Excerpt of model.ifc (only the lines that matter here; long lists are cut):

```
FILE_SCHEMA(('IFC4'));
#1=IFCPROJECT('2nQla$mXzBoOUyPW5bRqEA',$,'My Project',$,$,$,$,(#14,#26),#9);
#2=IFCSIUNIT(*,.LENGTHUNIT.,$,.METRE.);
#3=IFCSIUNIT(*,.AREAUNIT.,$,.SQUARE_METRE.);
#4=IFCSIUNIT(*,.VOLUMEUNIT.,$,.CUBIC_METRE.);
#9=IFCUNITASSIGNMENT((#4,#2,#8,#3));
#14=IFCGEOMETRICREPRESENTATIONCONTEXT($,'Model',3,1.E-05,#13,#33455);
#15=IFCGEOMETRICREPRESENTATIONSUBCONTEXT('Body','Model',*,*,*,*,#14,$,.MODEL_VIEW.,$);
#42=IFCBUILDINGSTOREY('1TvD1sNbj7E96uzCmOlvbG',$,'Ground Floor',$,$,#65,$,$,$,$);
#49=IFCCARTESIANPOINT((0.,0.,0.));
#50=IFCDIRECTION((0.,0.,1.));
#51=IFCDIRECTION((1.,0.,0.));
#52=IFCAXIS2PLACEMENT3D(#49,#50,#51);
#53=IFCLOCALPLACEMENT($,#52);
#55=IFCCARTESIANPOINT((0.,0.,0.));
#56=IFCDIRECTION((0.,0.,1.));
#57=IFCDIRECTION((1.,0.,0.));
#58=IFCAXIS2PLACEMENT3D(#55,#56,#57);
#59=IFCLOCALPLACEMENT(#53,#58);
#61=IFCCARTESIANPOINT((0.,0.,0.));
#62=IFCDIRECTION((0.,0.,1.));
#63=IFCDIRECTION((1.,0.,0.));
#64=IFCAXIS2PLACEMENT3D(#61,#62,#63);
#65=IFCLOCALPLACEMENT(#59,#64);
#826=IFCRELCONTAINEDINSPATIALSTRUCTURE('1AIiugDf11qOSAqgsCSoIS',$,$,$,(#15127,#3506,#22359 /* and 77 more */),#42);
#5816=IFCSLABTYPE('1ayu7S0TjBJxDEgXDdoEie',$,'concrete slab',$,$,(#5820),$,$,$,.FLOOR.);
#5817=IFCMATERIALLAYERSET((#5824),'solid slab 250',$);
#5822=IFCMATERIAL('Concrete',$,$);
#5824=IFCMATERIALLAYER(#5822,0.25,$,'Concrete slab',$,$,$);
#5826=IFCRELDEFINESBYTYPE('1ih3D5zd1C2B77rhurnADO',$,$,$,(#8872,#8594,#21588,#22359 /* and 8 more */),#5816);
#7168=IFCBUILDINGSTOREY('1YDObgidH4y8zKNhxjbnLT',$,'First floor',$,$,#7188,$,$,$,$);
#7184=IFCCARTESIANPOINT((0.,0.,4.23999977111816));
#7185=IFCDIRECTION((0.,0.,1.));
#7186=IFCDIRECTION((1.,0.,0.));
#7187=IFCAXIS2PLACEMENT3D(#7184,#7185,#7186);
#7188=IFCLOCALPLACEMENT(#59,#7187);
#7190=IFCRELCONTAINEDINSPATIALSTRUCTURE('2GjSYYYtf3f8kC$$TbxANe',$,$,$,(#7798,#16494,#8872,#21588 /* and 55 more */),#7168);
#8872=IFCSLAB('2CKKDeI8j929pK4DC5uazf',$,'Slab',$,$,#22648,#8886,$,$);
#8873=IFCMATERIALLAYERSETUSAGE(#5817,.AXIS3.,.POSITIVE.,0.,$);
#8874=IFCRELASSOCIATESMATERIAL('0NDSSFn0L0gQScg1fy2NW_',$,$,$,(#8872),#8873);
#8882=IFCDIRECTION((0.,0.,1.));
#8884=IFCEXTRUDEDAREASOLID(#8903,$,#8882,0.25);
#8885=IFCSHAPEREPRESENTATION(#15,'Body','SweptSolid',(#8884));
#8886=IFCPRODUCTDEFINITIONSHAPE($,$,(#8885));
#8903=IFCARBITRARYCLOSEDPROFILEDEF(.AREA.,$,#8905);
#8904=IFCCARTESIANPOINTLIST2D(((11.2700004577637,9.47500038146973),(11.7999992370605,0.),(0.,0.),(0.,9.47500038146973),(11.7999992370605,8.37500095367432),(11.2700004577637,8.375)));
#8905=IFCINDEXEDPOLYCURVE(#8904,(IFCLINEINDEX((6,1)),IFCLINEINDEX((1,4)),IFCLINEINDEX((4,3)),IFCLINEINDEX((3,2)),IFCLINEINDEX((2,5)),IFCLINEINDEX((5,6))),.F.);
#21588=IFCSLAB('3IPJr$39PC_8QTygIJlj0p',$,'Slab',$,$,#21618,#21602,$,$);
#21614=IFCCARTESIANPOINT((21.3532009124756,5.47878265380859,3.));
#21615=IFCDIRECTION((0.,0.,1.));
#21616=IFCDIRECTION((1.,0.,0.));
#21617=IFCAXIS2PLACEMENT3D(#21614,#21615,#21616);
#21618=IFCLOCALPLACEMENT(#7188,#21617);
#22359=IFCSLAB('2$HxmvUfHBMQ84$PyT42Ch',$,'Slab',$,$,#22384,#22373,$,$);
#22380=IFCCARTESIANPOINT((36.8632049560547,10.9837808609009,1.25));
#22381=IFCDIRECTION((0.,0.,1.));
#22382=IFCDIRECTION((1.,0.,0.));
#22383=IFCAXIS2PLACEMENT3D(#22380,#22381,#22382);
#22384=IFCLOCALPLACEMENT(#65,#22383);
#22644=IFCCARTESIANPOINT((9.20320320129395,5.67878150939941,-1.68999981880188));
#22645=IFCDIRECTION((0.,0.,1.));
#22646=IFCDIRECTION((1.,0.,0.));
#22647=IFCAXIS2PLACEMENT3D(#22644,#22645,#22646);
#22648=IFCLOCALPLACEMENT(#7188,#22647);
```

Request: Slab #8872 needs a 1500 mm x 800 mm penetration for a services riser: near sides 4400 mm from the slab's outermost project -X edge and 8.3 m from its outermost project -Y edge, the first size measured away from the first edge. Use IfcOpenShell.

```python
import numpy as np
import ifcopenshell
import ifcopenshell.api.feature
import ifcopenshell.api.geometry
import ifcopenshell.api.root
import ifcopenshell.geom
import ifcopenshell.util.placement
import ifcopenshell.util.representation
import ifcopenshell.util.shape
import ifcopenshell.util.unit

model = ifcopenshell.open("model.ifc")
unit_scale = ifcopenshell.util.unit.calculate_unit_scale(model)
settings = ifcopenshell.geom.settings()


def volume(element):
    """Net volume in cubic metres, openings subtracted."""
    shape = ifcopenshell.geom.create_shape(settings, element)
    return ifcopenshell.util.shape.get_volume(shape.geometry)


slab = model.by_id(8872)
before = volume(slab)

# Extent in the slab's own axes, in metres. The edges named are its -X and -Y sides.
slab_shape = ifcopenshell.geom.create_shape(settings, slab)
vertices = ifcopenshell.util.shape.get_vertices(slab_shape.geometry)
x_min, y_min, bottom = vertices.min(axis=0)
top = vertices[:, 2].max()

opening = ifcopenshell.api.root.create_entity(model, ifc_class="IfcOpeningElement", name="Services riser opening", predefined_type="OPENING")
context = ifcopenshell.util.representation.get_context(model, "Model", "Body", "MODEL_VIEW")
width, depth = 1.5, 0.8
outline = [(0.0, 0.0), (width, 0.0), (width, depth), (0.0, depth), (0.0, 0.0)]
# Overshoot both faces by 50 mm so the cut is clean.
shape = ifcopenshell.api.geometry.add_slab_representation(
    model, context=context, depth=top - bottom + 0.1, polyline=outline
)
ifcopenshell.api.geometry.assign_representation(model, product=opening, representation=shape)

matrix = ifcopenshell.util.placement.get_local_placement(slab.ObjectPlacement)
matrix[:, 3] = matrix @ np.append(np.array([x_min + 4.4, y_min + 8.3, bottom - 0.05]) / unit_scale, 1.0)
ifcopenshell.api.geometry.edit_object_placement(model, product=opening, matrix=matrix, is_si=False)
ifcopenshell.api.feature.add_feature(model, feature=opening, element=slab)

after = volume(slab)

print(f"slab volume {before:.3f} -> {after:.3f} m3")

model.write("model_updated.ifc")
```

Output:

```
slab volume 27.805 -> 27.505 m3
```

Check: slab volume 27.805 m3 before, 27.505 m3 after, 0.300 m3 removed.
